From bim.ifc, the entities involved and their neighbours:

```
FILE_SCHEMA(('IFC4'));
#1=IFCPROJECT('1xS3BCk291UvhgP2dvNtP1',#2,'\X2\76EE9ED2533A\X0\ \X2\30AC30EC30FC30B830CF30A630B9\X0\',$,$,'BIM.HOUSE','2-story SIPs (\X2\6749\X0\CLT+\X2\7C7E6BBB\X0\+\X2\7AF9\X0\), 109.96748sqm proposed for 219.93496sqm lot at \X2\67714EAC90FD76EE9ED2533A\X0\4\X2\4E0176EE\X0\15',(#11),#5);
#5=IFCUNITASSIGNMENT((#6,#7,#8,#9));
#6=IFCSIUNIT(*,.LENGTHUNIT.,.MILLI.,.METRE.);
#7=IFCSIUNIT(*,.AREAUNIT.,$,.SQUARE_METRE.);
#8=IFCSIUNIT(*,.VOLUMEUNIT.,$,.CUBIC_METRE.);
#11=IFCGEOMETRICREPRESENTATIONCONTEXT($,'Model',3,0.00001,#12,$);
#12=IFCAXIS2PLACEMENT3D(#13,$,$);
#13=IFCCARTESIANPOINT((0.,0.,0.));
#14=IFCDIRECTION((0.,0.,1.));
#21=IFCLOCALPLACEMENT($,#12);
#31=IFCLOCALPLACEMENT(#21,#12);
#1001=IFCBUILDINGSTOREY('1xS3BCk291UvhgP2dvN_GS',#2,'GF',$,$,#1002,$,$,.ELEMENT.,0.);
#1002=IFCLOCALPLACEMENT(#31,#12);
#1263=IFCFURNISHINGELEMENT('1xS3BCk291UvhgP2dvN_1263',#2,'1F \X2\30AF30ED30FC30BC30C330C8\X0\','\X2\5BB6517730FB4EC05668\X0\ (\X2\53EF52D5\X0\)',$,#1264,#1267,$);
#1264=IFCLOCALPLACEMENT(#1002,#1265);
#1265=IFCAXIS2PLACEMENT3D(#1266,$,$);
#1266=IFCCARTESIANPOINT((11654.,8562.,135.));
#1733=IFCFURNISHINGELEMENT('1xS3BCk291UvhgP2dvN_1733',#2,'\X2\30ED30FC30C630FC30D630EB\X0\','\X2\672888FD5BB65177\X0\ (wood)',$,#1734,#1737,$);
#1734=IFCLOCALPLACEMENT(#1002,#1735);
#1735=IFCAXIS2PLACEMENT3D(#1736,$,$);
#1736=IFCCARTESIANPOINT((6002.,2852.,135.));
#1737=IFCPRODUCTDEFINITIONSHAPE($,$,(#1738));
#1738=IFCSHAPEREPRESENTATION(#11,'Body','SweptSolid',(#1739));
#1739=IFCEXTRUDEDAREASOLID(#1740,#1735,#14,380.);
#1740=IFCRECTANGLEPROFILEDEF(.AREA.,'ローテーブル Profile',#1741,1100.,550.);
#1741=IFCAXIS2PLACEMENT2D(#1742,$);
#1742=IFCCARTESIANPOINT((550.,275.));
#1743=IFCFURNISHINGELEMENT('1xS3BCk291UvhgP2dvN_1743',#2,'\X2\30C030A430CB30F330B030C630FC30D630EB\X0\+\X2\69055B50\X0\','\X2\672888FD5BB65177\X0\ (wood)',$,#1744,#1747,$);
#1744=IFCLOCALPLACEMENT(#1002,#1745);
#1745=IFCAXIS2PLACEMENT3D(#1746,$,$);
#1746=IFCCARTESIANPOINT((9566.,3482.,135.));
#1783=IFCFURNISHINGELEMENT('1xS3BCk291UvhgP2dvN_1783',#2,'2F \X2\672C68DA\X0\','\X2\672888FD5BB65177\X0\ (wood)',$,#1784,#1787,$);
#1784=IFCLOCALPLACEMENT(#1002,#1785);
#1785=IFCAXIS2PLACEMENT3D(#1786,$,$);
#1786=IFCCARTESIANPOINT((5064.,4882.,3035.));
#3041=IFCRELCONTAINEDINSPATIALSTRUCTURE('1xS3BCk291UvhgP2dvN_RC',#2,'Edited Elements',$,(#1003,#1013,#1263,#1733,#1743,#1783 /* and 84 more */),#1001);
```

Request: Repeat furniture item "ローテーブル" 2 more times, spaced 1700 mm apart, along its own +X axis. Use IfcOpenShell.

```python
import ifcopenshell
import ifcopenshell.api.geometry
import ifcopenshell.api.root
import ifcopenshell.util.element
import ifcopenshell.util.placement
import ifcopenshell.util.unit

model = ifcopenshell.open("bim.ifc")
unit_scale = ifcopenshell.util.unit.calculate_unit_scale(model)


def reuse_history(source, copy):
    """copy_class also copies each property set's owner history, people and application; keep the originals."""
    for rel in copy.IsDefinedBy:
        if rel.is_a("IfcRelDefinesByProperties") and (history := rel.RelatingPropertyDefinition.OwnerHistory):
            rel.RelatingPropertyDefinition.OwnerHistory = source.OwnerHistory
            ifcopenshell.util.element.remove_deep2(model, history)


source = model.by_guid("1xS3BCk291UvhgP2dvN_1733")
base = ifcopenshell.util.placement.get_local_placement(source.ObjectPlacement)
step = base[:3, 0] * 1.7 / unit_scale

for i in range(1, 3):
    copy = ifcopenshell.api.root.copy_class(model, product=source)
    copy.Representation = ifcopenshell.util.element.copy_deep(
        model, source.Representation, exclude=["IfcGeometricRepresentationContext", "IfcRepresentationMap"]
    )
    reuse_history(source, copy)
    matrix = base.copy()
    matrix[:3, 3] += i * step
    print("added at", matrix[:3, 3].round(3) + 0.0)
    ifcopenshell.api.geometry.edit_object_placement(model, product=copy, matrix=matrix, is_si=False)

model.write("bim-out.ifc")
```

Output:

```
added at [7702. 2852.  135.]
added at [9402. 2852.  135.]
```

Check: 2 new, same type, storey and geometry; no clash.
